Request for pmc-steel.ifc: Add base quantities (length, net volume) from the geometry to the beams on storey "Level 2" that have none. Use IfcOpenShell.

First a look at what the model holds.

```python
import ifcopenshell
import ifcopenshell.util.element
import ifcopenshell.util.unit

model = ifcopenshell.open("pmc-steel.ifc")
print(model.schema)
for unit_type in ("LENGTHUNIT", "AREAUNIT", "VOLUMEUNIT"):
    print(unit_type, ifcopenshell.util.unit.calculate_unit_scale(model, unit_type))
storey = next(s for s in model.by_type("IfcBuildingStorey") if s.Name == "Level 2")
beams = [e for e in ifcopenshell.util.element.get_decomposition(storey) if e.is_a("IfcBeam")]
for e in sorted(beams, key=lambda e: e.id()):
    print(e.id(), e.is_a(), e.Name, list(ifcopenshell.util.element.get_psets(e, qtos_only=True)), sep=" | ")
```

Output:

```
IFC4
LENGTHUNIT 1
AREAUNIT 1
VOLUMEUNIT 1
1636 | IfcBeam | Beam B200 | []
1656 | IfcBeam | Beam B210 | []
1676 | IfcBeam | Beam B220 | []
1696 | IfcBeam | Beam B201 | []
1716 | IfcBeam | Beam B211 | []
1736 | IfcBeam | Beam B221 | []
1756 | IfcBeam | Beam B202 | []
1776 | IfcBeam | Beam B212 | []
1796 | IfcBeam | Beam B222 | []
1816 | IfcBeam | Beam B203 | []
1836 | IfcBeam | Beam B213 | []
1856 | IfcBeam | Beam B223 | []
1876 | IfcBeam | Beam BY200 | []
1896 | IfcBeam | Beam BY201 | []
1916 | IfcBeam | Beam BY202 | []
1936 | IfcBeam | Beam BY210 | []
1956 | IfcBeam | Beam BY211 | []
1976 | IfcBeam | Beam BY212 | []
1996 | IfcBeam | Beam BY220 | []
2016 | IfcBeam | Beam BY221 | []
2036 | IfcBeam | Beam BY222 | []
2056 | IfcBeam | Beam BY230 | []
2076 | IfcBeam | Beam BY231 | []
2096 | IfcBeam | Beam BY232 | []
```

```python
import ifcopenshell
import ifcopenshell.api.pset
import ifcopenshell.geom
import ifcopenshell.util.element
import ifcopenshell.util.shape
import ifcopenshell.util.unit

model = ifcopenshell.open("pmc-steel.ifc")
unit_scale = ifcopenshell.util.unit.calculate_unit_scale(model)
volume_scale = ifcopenshell.util.unit.calculate_unit_scale(model, "VOLUMEUNIT")
settings = ifcopenshell.geom.settings()

storey = next(s for s in model.by_type("IfcBuildingStorey") if s.Name == "Level 2")
beams = [e for e in ifcopenshell.util.element.get_decomposition(storey) if e.is_a("IfcBeam")]

for e in sorted(beams, key=lambda e: e.id()):
    if ifcopenshell.util.element.get_psets(e, qtos_only=True, should_inherit=False):
        continue
    # Geometry comes back in metres, in the element's own axes.
    shape = ifcopenshell.geom.create_shape(settings, e)
    values = {
        "Length": ifcopenshell.util.shape.get_max_xyz(shape.geometry) / unit_scale,
        "NetVolume": ifcopenshell.util.shape.get_volume(shape.geometry) / volume_scale,
    }
    qto = ifcopenshell.api.pset.add_qto(model, product=e, name="Qto_BeamBaseQuantities")
    ifcopenshell.api.pset.edit_qto(model, qto=qto, properties=values)
    print(e.id(), {k: round(v, 3) for k, v in values.items()})

model.write("pmc-steel_updated.ifc")
```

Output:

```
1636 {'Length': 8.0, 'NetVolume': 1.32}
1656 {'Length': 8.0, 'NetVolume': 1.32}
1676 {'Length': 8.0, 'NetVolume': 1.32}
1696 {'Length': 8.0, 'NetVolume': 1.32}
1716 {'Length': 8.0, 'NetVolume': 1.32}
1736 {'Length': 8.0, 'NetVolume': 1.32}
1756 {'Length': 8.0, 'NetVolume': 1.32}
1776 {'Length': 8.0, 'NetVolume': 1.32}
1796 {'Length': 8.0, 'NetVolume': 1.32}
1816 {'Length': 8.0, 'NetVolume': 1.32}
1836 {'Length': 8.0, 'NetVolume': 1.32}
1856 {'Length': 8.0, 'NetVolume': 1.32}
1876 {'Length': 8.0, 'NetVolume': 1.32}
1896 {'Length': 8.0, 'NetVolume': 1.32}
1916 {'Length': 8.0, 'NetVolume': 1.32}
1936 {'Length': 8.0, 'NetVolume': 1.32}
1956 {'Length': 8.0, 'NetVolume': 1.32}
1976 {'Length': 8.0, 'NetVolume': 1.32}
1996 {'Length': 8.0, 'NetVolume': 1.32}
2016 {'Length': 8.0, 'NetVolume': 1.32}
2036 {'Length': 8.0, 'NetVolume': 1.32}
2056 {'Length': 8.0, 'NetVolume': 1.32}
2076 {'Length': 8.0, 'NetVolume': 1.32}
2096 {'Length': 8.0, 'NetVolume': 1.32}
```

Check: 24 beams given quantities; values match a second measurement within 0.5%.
